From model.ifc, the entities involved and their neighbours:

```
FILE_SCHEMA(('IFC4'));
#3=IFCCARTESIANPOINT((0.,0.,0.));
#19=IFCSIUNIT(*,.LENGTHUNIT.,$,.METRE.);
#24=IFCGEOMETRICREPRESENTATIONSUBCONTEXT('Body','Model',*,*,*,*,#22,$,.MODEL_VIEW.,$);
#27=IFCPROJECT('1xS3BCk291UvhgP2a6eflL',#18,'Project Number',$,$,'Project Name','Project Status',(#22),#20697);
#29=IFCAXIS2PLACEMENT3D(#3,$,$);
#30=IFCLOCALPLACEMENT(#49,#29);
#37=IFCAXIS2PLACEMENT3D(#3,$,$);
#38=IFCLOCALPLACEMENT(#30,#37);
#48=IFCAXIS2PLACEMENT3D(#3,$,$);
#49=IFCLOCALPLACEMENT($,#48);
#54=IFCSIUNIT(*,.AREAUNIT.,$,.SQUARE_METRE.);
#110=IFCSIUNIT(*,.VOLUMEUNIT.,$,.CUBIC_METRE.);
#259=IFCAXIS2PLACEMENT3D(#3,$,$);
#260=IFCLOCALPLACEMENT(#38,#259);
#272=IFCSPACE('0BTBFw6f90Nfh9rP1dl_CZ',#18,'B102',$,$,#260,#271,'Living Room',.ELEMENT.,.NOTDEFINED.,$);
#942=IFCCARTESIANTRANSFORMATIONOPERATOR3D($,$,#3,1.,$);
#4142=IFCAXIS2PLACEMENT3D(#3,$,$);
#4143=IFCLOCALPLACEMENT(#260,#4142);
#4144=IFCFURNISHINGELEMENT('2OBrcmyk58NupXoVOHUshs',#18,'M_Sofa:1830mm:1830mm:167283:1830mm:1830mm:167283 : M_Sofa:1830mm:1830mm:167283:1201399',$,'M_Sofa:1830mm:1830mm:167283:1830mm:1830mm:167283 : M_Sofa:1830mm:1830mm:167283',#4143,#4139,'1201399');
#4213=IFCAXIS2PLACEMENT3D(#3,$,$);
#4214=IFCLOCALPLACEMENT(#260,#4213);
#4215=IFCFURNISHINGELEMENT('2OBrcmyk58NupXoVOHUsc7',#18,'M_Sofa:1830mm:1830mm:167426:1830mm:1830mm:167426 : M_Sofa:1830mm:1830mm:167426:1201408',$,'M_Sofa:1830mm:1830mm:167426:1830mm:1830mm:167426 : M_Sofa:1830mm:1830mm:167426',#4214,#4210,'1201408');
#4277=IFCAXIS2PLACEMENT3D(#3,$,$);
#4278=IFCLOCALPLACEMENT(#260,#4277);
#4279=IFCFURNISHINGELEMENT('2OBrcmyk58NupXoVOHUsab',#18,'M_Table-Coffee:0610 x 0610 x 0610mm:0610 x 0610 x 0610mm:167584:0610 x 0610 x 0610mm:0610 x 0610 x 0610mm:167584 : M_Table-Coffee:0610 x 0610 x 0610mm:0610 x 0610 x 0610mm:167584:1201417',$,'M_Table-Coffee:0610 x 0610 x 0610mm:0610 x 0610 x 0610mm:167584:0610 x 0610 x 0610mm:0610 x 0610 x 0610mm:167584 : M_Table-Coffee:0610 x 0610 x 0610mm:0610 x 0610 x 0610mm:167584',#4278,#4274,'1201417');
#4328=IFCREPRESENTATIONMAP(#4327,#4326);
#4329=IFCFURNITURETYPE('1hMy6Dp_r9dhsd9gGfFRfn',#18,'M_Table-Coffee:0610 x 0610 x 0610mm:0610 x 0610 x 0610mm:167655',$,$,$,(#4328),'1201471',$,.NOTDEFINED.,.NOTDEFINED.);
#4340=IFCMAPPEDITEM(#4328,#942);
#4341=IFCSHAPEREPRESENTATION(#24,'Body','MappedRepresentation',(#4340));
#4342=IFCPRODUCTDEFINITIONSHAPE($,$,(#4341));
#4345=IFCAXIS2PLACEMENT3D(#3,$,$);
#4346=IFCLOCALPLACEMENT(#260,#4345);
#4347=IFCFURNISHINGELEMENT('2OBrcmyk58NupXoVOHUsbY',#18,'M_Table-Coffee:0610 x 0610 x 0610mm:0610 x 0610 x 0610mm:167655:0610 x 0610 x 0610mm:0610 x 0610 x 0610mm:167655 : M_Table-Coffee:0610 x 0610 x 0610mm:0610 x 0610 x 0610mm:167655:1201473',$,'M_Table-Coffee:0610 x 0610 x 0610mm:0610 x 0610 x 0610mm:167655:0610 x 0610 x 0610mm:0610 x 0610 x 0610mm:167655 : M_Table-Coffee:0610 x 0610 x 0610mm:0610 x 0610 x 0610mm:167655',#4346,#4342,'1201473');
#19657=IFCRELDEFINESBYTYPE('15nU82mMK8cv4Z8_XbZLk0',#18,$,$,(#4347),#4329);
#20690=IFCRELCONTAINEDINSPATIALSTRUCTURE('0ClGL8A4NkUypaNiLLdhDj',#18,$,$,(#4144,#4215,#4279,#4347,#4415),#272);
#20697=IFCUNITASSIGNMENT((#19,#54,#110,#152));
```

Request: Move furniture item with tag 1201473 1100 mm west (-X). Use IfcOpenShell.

```python
import ifcopenshell
import ifcopenshell.api.geometry
import ifcopenshell.util.placement
import ifcopenshell.util.unit

model = ifcopenshell.open("model.ifc")
unit_scale = ifcopenshell.util.unit.calculate_unit_scale(model)

item = model.by_guid("2OBrcmyk58NupXoVOHUsbY")
matrix = ifcopenshell.util.placement.get_local_placement(item.ObjectPlacement)
matrix[0, 3] -= 1.1 / unit_scale
ifcopenshell.api.geometry.edit_object_placement(model, product=item, matrix=matrix, is_si=False)

print(ifcopenshell.util.placement.get_local_placement(item.ObjectPlacement).round(3) + 0.0)

model.write("model-out.ifc")
```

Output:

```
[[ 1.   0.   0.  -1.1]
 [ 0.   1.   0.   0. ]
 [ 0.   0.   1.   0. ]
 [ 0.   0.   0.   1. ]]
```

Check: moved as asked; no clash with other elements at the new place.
